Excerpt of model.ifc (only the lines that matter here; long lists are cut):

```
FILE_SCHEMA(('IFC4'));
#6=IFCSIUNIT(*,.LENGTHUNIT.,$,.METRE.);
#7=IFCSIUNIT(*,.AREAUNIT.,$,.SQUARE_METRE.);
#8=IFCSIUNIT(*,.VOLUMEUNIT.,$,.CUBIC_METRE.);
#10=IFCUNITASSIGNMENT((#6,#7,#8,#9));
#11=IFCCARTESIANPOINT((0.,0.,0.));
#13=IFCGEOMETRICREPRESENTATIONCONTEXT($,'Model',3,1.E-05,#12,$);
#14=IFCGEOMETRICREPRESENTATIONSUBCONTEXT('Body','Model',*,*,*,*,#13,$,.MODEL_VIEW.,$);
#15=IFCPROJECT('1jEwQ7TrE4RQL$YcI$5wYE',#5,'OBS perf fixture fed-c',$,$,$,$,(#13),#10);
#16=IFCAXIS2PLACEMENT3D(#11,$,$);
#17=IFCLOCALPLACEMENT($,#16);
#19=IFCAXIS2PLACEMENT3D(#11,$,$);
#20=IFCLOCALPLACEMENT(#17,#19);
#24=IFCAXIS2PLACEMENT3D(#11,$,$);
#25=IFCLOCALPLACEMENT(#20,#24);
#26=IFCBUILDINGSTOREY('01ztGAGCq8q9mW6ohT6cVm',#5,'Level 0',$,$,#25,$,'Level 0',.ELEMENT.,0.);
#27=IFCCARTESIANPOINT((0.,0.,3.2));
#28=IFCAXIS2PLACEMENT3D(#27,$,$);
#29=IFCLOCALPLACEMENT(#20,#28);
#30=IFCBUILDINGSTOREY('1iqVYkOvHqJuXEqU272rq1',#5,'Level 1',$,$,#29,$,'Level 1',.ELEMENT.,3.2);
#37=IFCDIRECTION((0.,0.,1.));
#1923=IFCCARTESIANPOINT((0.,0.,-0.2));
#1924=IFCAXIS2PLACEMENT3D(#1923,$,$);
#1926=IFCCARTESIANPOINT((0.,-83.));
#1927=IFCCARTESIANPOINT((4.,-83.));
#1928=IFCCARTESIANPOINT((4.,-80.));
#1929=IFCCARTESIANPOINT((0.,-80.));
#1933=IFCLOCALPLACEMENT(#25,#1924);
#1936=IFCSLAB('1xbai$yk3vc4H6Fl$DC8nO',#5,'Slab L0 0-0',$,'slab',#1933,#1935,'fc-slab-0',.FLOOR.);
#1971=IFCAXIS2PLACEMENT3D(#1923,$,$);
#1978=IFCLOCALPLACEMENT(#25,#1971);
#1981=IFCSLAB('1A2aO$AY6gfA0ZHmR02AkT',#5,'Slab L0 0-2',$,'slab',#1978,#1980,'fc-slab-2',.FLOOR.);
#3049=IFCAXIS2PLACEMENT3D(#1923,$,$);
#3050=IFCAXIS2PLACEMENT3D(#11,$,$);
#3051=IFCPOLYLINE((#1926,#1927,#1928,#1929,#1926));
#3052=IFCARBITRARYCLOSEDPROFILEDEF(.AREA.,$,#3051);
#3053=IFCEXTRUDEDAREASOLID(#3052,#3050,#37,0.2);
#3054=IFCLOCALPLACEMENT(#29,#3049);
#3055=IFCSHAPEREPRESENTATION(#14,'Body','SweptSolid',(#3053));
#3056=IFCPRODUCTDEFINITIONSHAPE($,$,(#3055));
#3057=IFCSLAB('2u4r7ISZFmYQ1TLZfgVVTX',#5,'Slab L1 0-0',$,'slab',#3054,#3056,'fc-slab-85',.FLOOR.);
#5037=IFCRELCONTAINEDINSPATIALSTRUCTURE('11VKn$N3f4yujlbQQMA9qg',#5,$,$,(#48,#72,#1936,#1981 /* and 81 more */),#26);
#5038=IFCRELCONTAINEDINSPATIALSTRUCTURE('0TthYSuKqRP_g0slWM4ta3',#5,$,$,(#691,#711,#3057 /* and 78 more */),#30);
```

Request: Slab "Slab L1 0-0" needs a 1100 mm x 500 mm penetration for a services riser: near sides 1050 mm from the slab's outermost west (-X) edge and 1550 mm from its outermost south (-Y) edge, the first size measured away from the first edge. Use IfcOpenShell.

```python
import numpy as np
import ifcopenshell
import ifcopenshell.api.feature
import ifcopenshell.api.geometry
import ifcopenshell.api.root
import ifcopenshell.geom
import ifcopenshell.util.placement
import ifcopenshell.util.representation
import ifcopenshell.util.shape
import ifcopenshell.util.unit

model = ifcopenshell.open("model.ifc")
unit_scale = ifcopenshell.util.unit.calculate_unit_scale(model)
settings = ifcopenshell.geom.settings()


def volume(element):
    """Net volume in cubic metres, openings subtracted."""
    shape = ifcopenshell.geom.create_shape(settings, element)
    return ifcopenshell.util.shape.get_volume(shape.geometry)


slab = model.by_id(3057)
before = volume(slab)

# Extent in the slab's own axes, in metres. The edges named are its -X and -Y sides.
slab_shape = ifcopenshell.geom.create_shape(settings, slab)
vertices = ifcopenshell.util.shape.get_vertices(slab_shape.geometry)
x_min, y_min, bottom = vertices.min(axis=0)
top = vertices[:, 2].max()

opening = ifcopenshell.api.root.create_entity(model, ifc_class="IfcOpeningElement", name="Services riser opening", predefined_type="OPENING")
context = ifcopenshell.util.representation.get_context(model, "Model", "Body", "MODEL_VIEW")
width, depth = 1.1, 0.5
outline = [(0.0, 0.0), (width, 0.0), (width, depth), (0.0, depth), (0.0, 0.0)]
# Overshoot both faces by 50 mm so the cut is clean.
shape = ifcopenshell.api.geometry.add_slab_representation(
    model, context=context, depth=top - bottom + 0.1, polyline=outline
)
ifcopenshell.api.geometry.assign_representation(model, product=opening, representation=shape)

matrix = ifcopenshell.util.placement.get_local_placement(slab.ObjectPlacement)
matrix[:, 3] = matrix @ np.append(np.array([x_min + 1.05, y_min + 1.55, bottom - 0.05]) / unit_scale, 1.0)
ifcopenshell.api.geometry.edit_object_placement(model, product=opening, matrix=matrix, is_si=False)
ifcopenshell.api.feature.add_feature(model, feature=opening, element=slab)

after = volume(slab)

print(f"slab volume {before:.3f} -> {after:.3f} m3")

model.write("model_v2.ifc")
```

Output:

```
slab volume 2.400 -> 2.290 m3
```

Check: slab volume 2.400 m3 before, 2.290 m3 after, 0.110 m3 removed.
